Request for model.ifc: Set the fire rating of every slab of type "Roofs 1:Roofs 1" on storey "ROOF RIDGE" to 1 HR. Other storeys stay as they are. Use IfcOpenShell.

First a look at what the model holds.

```python
import ifcopenshell
import ifcopenshell.util.element

model = ifcopenshell.open("model.ifc")
print(model.schema)
storey = next(s for s in model.by_type("IfcBuildingStorey") if s.Name == "ROOF RIDGE")
slabs = [e for e in ifcopenshell.util.element.get_decomposition(storey) if e.is_a("IfcSlab")]
seen = {}
for e in slabs:
    element_type = ifcopenshell.util.element.get_type(e)
    key = (element_type.Name if element_type != e and element_type else None, ifcopenshell.util.element.get_pset(e, "Pset_SlabCommon", "FireRating"))
    seen[key] = seen.get(key, 0) + 1
for (name, value), count in sorted(seen.items(), key=str):
    print(count, "x", name, "|", value)
```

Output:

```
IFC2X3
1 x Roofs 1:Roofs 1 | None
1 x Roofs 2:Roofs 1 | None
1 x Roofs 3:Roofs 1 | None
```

```python
import ifcopenshell
import ifcopenshell.api.pset
import ifcopenshell.util.element

model = ifcopenshell.open("model.ifc")

storey = next(s for s in model.by_type("IfcBuildingStorey") if s.Name == "ROOF RIDGE")
slabs = [e for e in ifcopenshell.util.element.get_decomposition(storey) if e.is_a("IfcSlab")]

count = 0
for e in slabs:
    element_type = ifcopenshell.util.element.get_type(e)
    if element_type in (None, e) or element_type.Name != "Roofs 1:Roofs 1":
        continue
    # add_pset returns the element's existing set when there is one.
    pset = ifcopenshell.api.pset.add_pset(model, product=e, name="Pset_SlabCommon")
    ifcopenshell.api.pset.edit_pset(model, pset=pset, properties={"FireRating": "1 HR"})
    count += 1

print(count, "slabs updated")

model.write("model-out.ifc")
```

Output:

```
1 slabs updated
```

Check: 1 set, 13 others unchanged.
